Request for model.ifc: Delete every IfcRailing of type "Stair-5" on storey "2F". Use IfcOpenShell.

First a look at what the model holds.

```python
import ifcopenshell
import ifcopenshell.util.element

model = ifcopenshell.open("model.ifc")
print(model.schema)
storey = next(s for s in model.by_type("IfcBuildingStorey") if s.Name == "2F")
railings = [e for e in ifcopenshell.util.element.get_decomposition(storey) if e.is_a("IfcRailing")]
seen = {}
for e in railings:
    element_type = ifcopenshell.util.element.get_type(e)
    name = element_type.Name if element_type not in (None, e) else None
    seen[name] = seen.get(name, 0) + 1
for name, count in sorted(seen.items(), key=str):
    print(count, "x", name)
```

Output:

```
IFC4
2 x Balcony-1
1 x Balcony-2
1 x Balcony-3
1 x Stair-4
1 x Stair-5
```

```python
import ifcopenshell
import ifcopenshell.api.root
import ifcopenshell.util.element

model = ifcopenshell.open("model.ifc")

storey = next(s for s in model.by_type("IfcBuildingStorey") if s.Name == "2F")
railings = [e for e in ifcopenshell.util.element.get_decomposition(storey) if e.is_a("IfcRailing")]
targets = [e for e in railings if (t := ifcopenshell.util.element.get_type(e)) not in (None, e) and t.Name == "Stair-5"]

for e in targets:
    ifcopenshell.api.root.remove_product(model, product=e)
print(len(targets), "removed")

model.write("model_v2.ifc")
```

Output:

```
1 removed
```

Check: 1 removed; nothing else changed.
